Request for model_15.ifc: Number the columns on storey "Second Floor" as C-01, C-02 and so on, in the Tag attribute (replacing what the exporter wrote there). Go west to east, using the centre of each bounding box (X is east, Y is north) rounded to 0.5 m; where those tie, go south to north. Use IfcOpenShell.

First a look at what the model holds.

```python
import ifcopenshell
import ifcopenshell.util.element
import ifcopenshell.util.placement

model = ifcopenshell.open("model_15.ifc")
print(model.schema)
storey = next(s for s in model.by_type("IfcBuildingStorey") if s.Name == "Second Floor")
columns = [e for e in ifcopenshell.util.element.get_decomposition(storey) if e.is_a("IfcColumn")]
for e in sorted(columns, key=lambda e: e.id()):
    origin = ifcopenshell.util.placement.get_local_placement(e.ObjectPlacement)[:3, 3]
    print(e.id(), e.Tag, e.Name, origin.round(2) + 0.0, sep=" | ")
```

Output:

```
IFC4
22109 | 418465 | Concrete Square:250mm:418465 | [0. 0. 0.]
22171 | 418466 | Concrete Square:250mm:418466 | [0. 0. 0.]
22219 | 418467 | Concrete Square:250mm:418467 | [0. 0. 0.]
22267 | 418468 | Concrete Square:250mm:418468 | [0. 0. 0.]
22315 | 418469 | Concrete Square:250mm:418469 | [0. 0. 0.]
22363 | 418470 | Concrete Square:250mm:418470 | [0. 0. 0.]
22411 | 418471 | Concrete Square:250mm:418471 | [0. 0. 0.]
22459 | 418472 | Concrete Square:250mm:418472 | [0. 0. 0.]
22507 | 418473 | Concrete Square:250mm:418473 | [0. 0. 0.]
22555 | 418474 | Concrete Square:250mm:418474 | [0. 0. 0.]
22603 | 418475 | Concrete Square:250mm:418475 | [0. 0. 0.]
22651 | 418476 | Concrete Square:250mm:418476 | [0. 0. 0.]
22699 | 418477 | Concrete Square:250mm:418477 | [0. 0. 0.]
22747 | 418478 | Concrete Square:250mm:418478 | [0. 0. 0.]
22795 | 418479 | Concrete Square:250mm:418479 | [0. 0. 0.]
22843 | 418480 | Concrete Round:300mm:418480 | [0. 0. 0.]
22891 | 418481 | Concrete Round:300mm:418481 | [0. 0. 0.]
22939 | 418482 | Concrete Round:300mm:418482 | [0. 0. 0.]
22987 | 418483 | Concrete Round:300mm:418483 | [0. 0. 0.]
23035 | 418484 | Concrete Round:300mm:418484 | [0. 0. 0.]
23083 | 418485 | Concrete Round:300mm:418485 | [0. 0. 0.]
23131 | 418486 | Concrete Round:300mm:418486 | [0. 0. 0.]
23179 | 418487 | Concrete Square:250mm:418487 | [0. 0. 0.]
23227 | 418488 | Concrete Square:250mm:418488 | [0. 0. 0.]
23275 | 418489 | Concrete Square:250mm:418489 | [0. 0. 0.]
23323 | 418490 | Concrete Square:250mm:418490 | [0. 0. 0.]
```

```python
import ifcopenshell
import ifcopenshell.geom
import ifcopenshell.util.element
import ifcopenshell.util.shape

model = ifcopenshell.open("model_15.ifc")
settings = ifcopenshell.geom.settings()
settings.set("use-world-coords", True)


def centre(element):
    shape = ifcopenshell.geom.create_shape(settings, element)
    return ifcopenshell.util.shape.get_bbox_centroid(shape.geometry)


storey = next(s for s in model.by_type("IfcBuildingStorey") if s.Name == "Second Floor")
columns = [e for e in ifcopenshell.util.element.get_decomposition(storey) if e.is_a("IfcColumn")]

# Insertion points can sit at a corner or the storey origin, so sort by the geometry (in metres).
centres = {e: centre(e) for e in columns}
columns.sort(key=lambda e: (round(centres[e][0] / 0.5), centres[e][1]))

for i, e in enumerate(columns, start=1):
    number = f"C-{i:02d}"
    e.Tag = number
    print(e.id(), number)

model.write("model_15_edited.ifc")
```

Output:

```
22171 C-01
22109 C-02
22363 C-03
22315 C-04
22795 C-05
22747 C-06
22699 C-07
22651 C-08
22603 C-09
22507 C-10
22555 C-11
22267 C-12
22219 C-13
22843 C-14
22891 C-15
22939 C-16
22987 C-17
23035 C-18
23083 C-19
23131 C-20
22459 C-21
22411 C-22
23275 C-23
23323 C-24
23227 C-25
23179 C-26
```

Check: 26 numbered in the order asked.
